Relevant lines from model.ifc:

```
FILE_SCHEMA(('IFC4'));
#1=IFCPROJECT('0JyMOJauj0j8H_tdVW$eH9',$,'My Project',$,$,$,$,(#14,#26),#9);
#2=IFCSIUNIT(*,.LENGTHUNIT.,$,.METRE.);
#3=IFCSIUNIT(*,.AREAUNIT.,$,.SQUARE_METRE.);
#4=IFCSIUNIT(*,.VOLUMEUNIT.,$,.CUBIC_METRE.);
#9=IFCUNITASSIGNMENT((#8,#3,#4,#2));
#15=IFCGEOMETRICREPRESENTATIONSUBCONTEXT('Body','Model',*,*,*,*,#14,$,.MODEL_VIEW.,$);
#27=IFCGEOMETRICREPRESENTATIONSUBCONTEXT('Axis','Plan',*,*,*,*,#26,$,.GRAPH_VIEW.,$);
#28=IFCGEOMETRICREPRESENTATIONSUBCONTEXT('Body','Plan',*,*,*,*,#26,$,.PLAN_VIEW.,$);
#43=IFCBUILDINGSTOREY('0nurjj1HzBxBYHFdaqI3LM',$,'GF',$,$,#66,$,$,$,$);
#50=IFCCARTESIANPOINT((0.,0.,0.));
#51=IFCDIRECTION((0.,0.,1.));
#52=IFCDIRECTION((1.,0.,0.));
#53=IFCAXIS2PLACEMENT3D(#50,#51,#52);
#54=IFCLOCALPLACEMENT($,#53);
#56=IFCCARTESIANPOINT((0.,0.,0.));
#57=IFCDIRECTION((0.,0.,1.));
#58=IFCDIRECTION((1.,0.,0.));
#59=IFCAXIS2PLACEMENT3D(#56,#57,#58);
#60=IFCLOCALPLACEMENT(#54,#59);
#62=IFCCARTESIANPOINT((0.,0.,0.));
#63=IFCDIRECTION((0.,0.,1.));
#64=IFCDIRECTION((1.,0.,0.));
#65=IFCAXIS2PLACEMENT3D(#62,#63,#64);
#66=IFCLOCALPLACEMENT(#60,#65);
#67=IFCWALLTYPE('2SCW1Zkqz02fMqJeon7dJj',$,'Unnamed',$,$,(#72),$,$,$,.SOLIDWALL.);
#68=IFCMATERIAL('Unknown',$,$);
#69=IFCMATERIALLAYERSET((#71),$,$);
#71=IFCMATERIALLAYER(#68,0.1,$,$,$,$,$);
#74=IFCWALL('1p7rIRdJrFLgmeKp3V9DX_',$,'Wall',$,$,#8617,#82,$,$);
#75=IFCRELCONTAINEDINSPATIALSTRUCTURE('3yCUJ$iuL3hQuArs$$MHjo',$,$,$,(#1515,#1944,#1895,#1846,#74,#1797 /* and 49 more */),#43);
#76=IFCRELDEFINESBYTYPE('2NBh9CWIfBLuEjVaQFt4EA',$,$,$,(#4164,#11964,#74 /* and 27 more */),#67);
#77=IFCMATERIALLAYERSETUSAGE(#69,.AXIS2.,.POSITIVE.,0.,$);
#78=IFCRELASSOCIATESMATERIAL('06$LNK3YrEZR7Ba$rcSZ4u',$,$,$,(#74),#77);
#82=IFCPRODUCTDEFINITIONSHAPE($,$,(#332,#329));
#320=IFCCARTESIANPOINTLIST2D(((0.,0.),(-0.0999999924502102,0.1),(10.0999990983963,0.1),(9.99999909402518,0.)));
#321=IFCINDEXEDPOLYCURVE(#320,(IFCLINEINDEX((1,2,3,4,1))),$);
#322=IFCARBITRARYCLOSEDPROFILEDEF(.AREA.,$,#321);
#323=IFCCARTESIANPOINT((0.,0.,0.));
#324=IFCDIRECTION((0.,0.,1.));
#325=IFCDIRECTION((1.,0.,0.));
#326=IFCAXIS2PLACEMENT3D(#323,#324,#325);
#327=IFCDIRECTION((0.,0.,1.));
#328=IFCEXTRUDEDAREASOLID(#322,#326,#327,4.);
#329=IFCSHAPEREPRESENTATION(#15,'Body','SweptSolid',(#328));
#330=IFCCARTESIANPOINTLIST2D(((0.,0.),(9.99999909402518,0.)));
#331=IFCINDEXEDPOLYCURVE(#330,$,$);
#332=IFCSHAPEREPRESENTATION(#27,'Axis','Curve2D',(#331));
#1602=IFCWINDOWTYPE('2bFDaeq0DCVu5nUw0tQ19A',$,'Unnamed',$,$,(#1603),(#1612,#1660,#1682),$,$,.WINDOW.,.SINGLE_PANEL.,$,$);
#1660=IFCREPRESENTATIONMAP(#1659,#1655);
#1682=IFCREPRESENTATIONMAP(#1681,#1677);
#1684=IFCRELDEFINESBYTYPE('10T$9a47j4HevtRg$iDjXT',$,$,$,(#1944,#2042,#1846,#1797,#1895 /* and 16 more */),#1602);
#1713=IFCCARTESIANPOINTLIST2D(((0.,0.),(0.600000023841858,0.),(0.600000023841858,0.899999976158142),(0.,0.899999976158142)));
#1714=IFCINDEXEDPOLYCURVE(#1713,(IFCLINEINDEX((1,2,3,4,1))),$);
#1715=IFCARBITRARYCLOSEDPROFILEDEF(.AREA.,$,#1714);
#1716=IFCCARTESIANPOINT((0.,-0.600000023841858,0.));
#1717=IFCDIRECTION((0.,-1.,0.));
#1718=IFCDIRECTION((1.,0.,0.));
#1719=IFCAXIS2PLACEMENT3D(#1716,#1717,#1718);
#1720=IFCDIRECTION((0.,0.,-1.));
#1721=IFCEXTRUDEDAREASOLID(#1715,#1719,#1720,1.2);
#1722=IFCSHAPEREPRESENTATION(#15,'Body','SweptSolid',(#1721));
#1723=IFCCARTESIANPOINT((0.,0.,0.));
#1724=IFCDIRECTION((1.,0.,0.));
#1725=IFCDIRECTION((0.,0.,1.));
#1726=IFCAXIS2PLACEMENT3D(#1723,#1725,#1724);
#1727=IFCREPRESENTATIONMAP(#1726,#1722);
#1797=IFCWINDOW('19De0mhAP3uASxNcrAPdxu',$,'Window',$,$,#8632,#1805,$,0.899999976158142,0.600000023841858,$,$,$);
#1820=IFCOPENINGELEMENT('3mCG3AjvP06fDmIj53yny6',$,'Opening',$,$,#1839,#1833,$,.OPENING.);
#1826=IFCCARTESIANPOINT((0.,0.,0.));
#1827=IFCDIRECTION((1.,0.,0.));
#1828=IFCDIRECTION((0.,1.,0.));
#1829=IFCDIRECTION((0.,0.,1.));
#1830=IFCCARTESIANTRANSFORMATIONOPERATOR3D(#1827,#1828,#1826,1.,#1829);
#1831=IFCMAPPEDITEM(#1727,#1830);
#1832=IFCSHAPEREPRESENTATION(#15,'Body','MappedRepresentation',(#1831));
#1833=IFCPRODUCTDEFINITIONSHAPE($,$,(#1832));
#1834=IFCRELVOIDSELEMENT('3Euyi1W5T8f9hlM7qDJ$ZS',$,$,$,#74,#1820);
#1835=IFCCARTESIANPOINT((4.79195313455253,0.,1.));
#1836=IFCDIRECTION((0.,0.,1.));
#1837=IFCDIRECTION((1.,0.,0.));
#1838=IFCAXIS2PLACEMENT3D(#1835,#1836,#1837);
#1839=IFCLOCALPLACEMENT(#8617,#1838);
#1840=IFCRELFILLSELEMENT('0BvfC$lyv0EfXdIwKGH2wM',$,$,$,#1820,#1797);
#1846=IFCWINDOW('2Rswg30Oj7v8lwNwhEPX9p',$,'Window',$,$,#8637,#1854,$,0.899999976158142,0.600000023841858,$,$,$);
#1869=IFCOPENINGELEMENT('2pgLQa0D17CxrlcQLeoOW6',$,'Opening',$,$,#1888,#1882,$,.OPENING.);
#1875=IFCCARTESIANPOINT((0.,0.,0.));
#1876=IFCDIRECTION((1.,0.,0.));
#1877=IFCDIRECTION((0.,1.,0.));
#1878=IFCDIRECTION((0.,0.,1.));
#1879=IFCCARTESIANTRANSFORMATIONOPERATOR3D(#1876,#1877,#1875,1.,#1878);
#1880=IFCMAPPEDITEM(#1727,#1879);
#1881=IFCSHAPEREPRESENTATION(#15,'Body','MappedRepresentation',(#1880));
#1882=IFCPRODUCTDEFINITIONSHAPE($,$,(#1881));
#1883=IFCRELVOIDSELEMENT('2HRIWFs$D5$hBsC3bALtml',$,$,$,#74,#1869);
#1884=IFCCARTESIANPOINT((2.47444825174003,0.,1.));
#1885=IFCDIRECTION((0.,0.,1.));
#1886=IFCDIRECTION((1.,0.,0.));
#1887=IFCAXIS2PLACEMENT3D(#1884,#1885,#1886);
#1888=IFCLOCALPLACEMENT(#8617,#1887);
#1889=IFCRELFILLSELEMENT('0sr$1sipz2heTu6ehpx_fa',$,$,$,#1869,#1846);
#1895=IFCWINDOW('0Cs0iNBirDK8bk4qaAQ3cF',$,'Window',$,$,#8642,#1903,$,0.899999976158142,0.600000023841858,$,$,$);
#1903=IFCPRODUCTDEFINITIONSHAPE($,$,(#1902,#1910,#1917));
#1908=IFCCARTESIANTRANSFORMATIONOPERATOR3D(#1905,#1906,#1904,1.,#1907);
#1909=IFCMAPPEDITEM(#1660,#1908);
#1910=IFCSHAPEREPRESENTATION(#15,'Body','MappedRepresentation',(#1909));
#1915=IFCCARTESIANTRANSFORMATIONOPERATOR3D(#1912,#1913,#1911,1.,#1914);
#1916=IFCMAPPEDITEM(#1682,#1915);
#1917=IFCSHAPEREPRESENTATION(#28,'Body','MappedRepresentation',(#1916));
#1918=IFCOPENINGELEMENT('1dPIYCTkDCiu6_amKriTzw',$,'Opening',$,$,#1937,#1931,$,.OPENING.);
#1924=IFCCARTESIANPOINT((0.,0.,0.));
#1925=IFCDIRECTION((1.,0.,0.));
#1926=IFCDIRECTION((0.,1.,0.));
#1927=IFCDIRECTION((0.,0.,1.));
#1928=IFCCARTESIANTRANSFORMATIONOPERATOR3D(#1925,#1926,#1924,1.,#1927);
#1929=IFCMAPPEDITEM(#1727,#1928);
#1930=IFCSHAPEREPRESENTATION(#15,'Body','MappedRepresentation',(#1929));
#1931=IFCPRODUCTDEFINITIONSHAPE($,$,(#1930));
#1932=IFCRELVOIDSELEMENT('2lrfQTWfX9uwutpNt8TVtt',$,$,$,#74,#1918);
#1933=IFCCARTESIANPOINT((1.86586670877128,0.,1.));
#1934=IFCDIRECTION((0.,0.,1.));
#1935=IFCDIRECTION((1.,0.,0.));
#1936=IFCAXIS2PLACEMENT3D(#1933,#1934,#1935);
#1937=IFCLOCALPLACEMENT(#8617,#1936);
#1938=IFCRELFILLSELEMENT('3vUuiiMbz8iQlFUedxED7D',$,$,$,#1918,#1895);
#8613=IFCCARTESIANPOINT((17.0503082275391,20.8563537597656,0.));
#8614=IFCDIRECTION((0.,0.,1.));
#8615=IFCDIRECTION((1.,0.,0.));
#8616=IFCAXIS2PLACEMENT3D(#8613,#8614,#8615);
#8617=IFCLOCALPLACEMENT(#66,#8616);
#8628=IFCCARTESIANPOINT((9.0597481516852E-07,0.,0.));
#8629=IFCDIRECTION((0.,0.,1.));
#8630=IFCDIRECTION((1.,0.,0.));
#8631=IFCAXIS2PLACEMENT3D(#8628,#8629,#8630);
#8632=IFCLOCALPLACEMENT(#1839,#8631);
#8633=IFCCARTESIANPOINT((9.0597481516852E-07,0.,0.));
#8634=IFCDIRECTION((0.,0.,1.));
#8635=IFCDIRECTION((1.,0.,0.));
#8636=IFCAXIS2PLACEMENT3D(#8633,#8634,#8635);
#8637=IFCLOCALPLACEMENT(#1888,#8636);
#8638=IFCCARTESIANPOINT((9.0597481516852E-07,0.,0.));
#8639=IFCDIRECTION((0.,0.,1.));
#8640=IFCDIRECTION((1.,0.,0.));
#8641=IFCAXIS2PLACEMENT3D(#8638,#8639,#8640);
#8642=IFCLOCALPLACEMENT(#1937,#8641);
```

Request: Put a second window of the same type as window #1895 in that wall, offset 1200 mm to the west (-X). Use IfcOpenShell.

```python
import ifcopenshell
import ifcopenshell.api.feature
import ifcopenshell.api.geometry
import ifcopenshell.api.root
import ifcopenshell.geom
import ifcopenshell.util.element
import ifcopenshell.util.placement
import ifcopenshell.util.shape

model = ifcopenshell.open("model.ifc")
settings = ifcopenshell.geom.settings()


def volume(element):
    """Net volume in cubic metres, openings subtracted."""
    shape = ifcopenshell.geom.create_shape(settings, element)
    return ifcopenshell.util.shape.get_volume(shape.geometry)


window = model.by_guid("0Cs0iNBirDK8bk4qaAQ3cF")
opening = window.FillsVoids[0].RelatingOpeningElement
wall = opening.VoidsElements[0].RelatingBuildingElement
before = volume(wall)
shift = ifcopenshell.util.placement.get_local_placement(wall.ObjectPlacement)[:3, 0] * -1.2

# copy_class copies the void relationship, type, container and properties, but no geometry.
new_opening = ifcopenshell.api.root.copy_class(model, product=opening)
new_opening.Representation = ifcopenshell.util.element.copy_deep(
    model, opening.Representation, exclude=["IfcGeometricRepresentationContext", "IfcRepresentationMap"]
)
new_window = ifcopenshell.api.root.copy_class(model, product=window)
new_window.Representation = ifcopenshell.util.element.copy_deep(
    model, window.Representation, exclude=["IfcGeometricRepresentationContext", "IfcRepresentationMap"]
)
ifcopenshell.api.feature.add_filling(model, opening=new_opening, element=new_window)

for old, new in ((opening, new_opening), (window, new_window)):
    matrix = ifcopenshell.util.placement.get_local_placement(old.ObjectPlacement)
    matrix[:3, 3] += shift
    ifcopenshell.api.geometry.edit_object_placement(model, product=new, matrix=matrix, is_si=False)

after = volume(wall)

print(f"wall volume {before:.3f} -> {after:.3f} m3")

model.write("model-out.ifc")
```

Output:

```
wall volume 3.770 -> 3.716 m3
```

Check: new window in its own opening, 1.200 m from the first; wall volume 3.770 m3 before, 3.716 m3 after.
